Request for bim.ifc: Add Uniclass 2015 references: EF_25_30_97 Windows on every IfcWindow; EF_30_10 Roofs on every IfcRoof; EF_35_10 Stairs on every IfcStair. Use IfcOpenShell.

First a look at what the model holds.

```python
import ifcopenshell

model = ifcopenshell.open("bim.ifc")
print(model.schema)
print("classifications:", [c.Name for c in model.by_type("IfcClassification")])
for ifc_class in ("IfcDoor", "IfcRoof", "IfcStair", "IfcWall", "IfcWindow"):
    print(ifc_class, len(model.by_type(ifc_class)))
```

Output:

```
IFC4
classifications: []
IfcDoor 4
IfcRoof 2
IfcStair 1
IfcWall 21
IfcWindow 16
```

```python
import ifcopenshell
import ifcopenshell.api.classification

model = ifcopenshell.open("bim.ifc")

system = ifcopenshell.api.classification.add_classification(model, classification="Uniclass 2015")

codes = {
    "IfcWindow": ("EF_25_30_97", "Windows"),
    "IfcRoof": ("EF_30_10", "Roofs"),
    "IfcStair": ("EF_35_10", "Stairs"),
}
for ifc_class, (code, name) in codes.items():
    products = model.by_type(ifc_class)
    ifcopenshell.api.classification.add_reference(
        model, products=products, classification=system, identification=code, name=name
    )
    print(code, len(products))

model.write("bim-out.ifc")
```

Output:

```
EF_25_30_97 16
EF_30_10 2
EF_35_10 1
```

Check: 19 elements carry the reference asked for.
